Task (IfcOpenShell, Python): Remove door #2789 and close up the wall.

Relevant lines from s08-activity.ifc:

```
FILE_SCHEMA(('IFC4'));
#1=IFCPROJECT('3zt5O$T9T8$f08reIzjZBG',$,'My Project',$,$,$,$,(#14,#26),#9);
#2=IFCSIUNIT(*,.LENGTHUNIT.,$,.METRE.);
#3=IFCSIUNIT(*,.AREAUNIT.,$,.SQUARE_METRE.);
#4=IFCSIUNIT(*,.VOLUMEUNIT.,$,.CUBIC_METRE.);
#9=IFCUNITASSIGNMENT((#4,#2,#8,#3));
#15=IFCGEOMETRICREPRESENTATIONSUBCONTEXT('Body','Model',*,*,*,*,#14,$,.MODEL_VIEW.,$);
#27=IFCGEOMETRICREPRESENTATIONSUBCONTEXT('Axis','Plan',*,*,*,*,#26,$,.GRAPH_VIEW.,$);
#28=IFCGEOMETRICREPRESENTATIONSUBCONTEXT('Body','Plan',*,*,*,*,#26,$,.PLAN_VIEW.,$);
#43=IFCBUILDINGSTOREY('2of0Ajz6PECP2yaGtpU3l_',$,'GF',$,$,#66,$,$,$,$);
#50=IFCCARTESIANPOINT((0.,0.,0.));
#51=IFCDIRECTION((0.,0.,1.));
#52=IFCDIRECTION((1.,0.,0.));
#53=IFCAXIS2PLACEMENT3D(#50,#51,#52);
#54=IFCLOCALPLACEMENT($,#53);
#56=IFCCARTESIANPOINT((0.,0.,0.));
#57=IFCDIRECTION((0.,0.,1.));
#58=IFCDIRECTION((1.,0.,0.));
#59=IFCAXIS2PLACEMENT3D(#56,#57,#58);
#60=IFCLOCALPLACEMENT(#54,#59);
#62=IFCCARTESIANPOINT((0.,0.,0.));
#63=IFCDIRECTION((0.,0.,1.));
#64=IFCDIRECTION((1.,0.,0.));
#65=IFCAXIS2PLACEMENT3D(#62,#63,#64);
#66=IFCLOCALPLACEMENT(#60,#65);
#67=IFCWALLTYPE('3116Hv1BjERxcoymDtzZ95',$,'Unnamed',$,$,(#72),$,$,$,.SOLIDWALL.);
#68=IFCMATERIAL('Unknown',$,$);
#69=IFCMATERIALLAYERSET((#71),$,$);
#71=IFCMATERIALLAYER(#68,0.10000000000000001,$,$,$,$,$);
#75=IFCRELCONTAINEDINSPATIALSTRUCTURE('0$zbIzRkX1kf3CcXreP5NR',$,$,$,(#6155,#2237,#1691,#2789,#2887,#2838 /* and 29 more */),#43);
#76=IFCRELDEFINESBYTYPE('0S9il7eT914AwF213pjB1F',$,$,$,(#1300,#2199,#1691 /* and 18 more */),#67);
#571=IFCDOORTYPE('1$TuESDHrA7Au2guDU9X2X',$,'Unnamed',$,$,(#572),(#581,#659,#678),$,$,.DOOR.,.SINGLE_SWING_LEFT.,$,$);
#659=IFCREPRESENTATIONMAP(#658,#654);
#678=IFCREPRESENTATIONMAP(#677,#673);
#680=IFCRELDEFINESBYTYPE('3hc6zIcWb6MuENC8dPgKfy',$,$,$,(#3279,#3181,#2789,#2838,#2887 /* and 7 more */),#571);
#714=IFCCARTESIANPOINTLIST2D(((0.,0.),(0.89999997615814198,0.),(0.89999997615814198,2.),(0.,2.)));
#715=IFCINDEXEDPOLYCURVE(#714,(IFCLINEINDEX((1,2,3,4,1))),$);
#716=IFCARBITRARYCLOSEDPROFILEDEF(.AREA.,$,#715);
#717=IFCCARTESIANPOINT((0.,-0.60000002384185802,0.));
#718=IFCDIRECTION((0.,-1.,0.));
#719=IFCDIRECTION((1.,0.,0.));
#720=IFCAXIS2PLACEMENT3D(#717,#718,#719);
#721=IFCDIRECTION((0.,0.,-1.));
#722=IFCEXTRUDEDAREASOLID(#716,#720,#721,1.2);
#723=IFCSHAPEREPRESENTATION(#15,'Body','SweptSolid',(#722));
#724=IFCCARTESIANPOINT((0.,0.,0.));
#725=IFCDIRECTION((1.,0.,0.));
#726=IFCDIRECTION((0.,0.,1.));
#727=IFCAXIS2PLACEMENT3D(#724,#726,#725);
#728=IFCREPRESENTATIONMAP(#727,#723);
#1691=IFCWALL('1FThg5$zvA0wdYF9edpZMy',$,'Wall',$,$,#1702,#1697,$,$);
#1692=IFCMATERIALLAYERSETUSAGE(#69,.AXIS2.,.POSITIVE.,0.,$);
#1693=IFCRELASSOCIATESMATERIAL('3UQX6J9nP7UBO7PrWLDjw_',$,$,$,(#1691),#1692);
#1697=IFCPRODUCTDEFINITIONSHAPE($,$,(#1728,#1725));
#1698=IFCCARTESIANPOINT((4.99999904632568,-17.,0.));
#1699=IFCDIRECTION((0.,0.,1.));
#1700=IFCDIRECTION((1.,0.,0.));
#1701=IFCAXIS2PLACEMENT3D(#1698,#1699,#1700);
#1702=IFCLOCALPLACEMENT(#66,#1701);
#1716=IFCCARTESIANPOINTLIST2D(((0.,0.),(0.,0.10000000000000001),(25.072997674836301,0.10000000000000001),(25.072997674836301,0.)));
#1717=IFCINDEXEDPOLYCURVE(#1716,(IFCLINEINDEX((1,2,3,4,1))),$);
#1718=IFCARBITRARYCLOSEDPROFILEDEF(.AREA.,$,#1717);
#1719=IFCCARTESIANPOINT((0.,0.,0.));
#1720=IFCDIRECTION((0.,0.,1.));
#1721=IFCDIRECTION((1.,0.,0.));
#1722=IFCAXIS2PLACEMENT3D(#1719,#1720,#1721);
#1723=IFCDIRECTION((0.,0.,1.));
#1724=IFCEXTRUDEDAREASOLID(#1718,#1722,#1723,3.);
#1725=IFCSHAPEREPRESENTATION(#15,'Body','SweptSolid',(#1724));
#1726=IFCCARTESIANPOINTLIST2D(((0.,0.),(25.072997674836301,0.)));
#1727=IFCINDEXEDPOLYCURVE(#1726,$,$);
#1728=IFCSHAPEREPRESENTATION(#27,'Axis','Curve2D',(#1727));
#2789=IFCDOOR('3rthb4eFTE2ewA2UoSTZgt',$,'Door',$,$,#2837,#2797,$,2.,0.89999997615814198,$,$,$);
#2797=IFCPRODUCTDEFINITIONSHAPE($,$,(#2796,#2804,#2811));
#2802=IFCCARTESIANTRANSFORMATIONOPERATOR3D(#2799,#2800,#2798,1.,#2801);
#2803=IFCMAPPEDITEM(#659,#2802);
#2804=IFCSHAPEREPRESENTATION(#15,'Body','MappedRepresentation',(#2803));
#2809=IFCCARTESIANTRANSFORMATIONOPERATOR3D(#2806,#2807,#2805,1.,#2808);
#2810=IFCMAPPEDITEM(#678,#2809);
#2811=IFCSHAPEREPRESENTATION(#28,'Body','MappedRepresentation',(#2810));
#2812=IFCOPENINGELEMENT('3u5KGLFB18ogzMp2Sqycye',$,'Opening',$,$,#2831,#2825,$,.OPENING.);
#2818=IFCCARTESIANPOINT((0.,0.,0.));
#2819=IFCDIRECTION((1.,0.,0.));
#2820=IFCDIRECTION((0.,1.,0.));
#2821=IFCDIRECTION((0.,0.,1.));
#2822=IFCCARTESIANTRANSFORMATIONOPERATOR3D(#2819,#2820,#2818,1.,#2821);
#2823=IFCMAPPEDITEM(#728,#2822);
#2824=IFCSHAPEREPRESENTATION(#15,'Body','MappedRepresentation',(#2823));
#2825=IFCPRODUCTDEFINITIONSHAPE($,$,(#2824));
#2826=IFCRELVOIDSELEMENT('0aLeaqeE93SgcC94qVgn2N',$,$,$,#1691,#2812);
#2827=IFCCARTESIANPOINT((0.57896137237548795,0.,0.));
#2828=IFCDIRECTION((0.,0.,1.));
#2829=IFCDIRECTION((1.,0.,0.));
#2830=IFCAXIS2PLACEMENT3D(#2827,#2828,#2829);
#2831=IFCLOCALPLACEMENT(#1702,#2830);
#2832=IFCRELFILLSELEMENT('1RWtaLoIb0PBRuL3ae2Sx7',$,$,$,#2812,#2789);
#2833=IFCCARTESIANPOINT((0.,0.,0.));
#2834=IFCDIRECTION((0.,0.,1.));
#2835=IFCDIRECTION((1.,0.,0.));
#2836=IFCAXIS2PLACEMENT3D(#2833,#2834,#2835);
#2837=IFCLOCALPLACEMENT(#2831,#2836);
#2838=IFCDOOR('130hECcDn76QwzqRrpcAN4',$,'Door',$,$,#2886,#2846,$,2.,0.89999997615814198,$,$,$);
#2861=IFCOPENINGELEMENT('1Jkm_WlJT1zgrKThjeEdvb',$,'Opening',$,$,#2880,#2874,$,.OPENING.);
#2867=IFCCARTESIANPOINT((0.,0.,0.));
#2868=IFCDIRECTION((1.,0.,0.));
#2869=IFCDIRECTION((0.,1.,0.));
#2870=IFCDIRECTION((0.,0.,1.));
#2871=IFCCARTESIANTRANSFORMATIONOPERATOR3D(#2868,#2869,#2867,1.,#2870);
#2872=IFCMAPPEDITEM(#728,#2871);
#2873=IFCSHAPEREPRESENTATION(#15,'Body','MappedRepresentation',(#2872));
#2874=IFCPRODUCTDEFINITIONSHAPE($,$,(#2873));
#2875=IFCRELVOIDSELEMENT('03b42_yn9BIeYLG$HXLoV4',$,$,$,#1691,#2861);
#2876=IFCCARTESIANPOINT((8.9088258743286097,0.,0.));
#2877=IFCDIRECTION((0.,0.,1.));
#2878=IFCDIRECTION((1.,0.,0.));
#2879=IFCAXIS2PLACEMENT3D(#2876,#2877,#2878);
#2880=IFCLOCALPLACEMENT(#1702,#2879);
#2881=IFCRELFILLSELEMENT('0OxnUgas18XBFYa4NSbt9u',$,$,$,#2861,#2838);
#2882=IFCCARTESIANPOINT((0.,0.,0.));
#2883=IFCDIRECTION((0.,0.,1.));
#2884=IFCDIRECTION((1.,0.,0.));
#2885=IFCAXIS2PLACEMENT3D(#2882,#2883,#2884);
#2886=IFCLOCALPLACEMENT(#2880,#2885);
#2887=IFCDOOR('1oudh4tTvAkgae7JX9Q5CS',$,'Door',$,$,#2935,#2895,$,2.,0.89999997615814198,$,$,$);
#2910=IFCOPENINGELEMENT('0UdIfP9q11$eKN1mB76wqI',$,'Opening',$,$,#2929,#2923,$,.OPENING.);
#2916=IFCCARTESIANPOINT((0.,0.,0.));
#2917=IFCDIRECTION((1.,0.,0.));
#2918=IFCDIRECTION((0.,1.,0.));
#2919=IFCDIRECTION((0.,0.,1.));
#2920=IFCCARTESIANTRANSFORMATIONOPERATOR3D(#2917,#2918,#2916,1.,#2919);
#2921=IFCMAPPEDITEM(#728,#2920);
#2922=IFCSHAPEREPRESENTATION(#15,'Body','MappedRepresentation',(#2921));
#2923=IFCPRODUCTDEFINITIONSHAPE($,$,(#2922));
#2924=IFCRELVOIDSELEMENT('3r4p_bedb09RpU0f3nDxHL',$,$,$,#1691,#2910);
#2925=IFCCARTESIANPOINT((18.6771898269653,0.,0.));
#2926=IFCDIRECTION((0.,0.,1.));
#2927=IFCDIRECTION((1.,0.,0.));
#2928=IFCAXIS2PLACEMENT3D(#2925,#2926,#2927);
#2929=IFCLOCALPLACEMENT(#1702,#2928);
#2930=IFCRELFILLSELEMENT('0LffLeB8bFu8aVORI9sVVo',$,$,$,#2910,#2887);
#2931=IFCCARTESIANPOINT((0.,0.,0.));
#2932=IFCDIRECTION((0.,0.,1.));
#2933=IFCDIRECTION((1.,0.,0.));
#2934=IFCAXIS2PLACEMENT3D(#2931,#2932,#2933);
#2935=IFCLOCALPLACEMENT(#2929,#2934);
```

```python
import ifcopenshell
import ifcopenshell.api.feature
import ifcopenshell.api.root
import ifcopenshell.geom
import ifcopenshell.util.shape

model = ifcopenshell.open("s08-activity.ifc")
settings = ifcopenshell.geom.settings()


def volume(element):
    """Net volume in cubic metres, openings subtracted."""
    shape = ifcopenshell.geom.create_shape(settings, element)
    return ifcopenshell.util.shape.get_volume(shape.geometry)


door = model.by_id(2789)
opening = door.FillsVoids[0].RelatingOpeningElement
wall = opening.VoidsElements[0].RelatingBuildingElement
before = volume(wall)

ifcopenshell.api.root.remove_product(model, product=door)
ifcopenshell.api.feature.remove_feature(model, feature=opening)

after = volume(wall)

print(f"wall volume {before:.3f} -> {after:.3f} m3")

model.write("s08-activity_edited.ifc")
```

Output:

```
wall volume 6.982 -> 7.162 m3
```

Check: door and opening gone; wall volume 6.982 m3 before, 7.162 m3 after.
